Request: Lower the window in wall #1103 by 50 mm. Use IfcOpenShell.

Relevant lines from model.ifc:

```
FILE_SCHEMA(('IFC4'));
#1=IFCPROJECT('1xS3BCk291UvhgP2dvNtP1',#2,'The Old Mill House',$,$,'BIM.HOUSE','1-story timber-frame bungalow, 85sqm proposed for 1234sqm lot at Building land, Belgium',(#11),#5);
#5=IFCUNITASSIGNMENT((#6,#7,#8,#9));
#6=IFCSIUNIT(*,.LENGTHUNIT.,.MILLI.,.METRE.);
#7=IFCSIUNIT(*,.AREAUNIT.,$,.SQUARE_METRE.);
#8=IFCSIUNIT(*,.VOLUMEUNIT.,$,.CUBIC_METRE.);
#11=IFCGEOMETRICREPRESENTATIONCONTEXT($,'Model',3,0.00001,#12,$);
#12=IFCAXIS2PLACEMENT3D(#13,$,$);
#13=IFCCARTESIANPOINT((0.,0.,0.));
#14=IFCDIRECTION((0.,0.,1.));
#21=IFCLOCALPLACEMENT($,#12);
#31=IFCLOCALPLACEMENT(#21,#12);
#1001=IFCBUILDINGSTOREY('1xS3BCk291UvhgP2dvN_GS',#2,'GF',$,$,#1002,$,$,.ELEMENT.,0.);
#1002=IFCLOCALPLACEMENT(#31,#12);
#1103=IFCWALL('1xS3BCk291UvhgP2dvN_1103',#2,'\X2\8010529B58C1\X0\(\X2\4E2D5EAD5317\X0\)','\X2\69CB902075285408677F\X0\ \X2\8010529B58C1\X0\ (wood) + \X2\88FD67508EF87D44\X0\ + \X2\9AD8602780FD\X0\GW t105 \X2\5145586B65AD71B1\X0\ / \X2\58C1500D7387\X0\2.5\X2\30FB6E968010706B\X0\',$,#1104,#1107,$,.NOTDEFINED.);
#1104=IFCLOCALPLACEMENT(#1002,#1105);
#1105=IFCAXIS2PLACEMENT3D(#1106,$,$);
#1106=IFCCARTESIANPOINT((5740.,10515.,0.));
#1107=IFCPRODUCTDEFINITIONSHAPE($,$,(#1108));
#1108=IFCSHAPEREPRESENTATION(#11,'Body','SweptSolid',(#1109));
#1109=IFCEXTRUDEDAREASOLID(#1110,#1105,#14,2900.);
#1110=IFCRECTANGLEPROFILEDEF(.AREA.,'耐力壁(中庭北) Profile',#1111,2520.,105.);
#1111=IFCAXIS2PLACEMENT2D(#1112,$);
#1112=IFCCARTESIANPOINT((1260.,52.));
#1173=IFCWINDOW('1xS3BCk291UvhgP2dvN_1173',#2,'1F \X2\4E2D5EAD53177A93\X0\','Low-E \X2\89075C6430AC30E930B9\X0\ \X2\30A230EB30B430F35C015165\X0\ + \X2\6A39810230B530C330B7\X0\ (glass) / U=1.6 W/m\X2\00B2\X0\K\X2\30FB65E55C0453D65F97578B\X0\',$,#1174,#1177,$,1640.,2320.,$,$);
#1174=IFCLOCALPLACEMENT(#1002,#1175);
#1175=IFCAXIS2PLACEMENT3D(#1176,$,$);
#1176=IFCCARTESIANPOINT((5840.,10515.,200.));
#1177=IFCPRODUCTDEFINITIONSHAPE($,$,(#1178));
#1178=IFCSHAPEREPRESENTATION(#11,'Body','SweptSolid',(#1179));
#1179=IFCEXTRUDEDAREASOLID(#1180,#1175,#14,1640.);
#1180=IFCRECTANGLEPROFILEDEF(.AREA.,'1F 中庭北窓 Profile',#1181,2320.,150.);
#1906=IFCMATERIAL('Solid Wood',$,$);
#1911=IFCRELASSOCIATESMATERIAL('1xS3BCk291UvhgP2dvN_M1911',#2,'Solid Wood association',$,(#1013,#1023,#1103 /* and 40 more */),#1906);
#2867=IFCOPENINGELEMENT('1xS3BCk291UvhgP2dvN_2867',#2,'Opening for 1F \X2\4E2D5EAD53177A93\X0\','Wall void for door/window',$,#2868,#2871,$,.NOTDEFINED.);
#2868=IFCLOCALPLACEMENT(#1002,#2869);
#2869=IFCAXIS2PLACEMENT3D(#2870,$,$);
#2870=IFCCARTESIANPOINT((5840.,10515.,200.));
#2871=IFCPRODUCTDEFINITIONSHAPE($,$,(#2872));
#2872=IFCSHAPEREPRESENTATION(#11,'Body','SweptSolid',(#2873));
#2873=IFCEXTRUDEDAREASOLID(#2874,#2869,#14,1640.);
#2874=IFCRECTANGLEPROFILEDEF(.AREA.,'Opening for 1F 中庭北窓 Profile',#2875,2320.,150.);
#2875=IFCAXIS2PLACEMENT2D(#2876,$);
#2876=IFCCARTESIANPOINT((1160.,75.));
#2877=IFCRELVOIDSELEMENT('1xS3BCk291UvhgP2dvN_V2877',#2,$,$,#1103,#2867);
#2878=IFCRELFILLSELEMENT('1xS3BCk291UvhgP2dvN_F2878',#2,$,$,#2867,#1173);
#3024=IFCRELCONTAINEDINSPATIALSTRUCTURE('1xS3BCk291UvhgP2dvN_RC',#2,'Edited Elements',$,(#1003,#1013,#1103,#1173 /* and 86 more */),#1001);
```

```python
import numpy as np
import ifcopenshell
import ifcopenshell.api.geometry
import ifcopenshell.util.placement
import ifcopenshell.util.unit

model = ifcopenshell.open("model.ifc")
unit_scale = ifcopenshell.util.unit.calculate_unit_scale(model)

window = model.by_guid("1xS3BCk291UvhgP2dvN_1173")
opening = window.FillsVoids[0].RelatingOpeningElement
dz = -0.05 / unit_scale

shift = np.array([0.0, 0.0, dz])
# The window is not placed relative to its opening, so move both.
for product in (opening, window):
    matrix = ifcopenshell.util.placement.get_local_placement(product.ObjectPlacement)
    matrix[:3, 3] += shift
    ifcopenshell.api.geometry.edit_object_placement(model, product=product, matrix=matrix, is_si=False)

print(f"moved by {dz * unit_scale:+.3f} m")

model.write("model_edited.ifc")
```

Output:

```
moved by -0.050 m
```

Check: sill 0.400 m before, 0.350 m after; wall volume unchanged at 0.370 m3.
